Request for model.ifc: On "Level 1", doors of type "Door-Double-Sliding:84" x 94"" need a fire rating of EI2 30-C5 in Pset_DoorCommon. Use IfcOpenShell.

First a look at what the model holds.

```python
import ifcopenshell
import ifcopenshell.util.element

model = ifcopenshell.open("model.ifc")
print(model.schema)
storey = next(s for s in model.by_type("IfcBuildingStorey") if s.Name == "Level 1")
doors = [e for e in ifcopenshell.util.element.get_decomposition(storey) if e.is_a("IfcDoor")]
seen = {}
for e in doors:
    element_type = ifcopenshell.util.element.get_type(e)
    key = (element_type.Name if element_type != e and element_type else None, ifcopenshell.util.element.get_pset(e, "Pset_DoorCommon", "FireRating"))
    seen[key] = seen.get(key, 0) + 1
for (name, value), count in sorted(seen.items(), key=str):
    print(count, "x", name, "|", value)
```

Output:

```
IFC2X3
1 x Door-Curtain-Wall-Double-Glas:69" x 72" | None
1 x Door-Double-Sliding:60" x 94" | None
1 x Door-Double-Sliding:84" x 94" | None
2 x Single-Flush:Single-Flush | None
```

```python
import ifcopenshell
import ifcopenshell.api.pset
import ifcopenshell.util.element

model = ifcopenshell.open("model.ifc")

storey = next(s for s in model.by_type("IfcBuildingStorey") if s.Name == "Level 1")
doors = [e for e in ifcopenshell.util.element.get_decomposition(storey) if e.is_a("IfcDoor")]

count = 0
for e in doors:
    element_type = ifcopenshell.util.element.get_type(e)
    if element_type in (None, e) or element_type.Name != 'Door-Double-Sliding:84" x 94"':
        continue
    # add_pset returns the element's existing set when there is one.
    pset = ifcopenshell.api.pset.add_pset(model, product=e, name="Pset_DoorCommon")
    ifcopenshell.api.pset.edit_pset(model, pset=pset, properties={"FireRating": "EI2 30-C5"})
    count += 1

print(count, "doors updated")

model.write("model-out.ifc")
```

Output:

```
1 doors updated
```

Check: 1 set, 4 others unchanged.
